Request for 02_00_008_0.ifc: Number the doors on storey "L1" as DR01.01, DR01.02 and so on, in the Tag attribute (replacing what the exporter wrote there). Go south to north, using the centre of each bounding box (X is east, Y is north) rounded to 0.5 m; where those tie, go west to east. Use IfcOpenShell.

First a look at what the model holds.

```python
import ifcopenshell
import ifcopenshell.util.element
import ifcopenshell.util.placement

model = ifcopenshell.open("02_00_008_0.ifc")
print(model.schema)
storey = next(s for s in model.by_type("IfcBuildingStorey") if s.Name == "L1")
doors = [e for e in ifcopenshell.util.element.get_decomposition(storey) if e.is_a("IfcDoor")]
for e in sorted(doors, key=lambda e: e.id()):
    origin = ifcopenshell.util.placement.get_local_placement(e.ObjectPlacement)[:3, 3]
    print(e.id(), e.Tag, e.Name, origin.round(2) + 0.0, sep=" | ")
```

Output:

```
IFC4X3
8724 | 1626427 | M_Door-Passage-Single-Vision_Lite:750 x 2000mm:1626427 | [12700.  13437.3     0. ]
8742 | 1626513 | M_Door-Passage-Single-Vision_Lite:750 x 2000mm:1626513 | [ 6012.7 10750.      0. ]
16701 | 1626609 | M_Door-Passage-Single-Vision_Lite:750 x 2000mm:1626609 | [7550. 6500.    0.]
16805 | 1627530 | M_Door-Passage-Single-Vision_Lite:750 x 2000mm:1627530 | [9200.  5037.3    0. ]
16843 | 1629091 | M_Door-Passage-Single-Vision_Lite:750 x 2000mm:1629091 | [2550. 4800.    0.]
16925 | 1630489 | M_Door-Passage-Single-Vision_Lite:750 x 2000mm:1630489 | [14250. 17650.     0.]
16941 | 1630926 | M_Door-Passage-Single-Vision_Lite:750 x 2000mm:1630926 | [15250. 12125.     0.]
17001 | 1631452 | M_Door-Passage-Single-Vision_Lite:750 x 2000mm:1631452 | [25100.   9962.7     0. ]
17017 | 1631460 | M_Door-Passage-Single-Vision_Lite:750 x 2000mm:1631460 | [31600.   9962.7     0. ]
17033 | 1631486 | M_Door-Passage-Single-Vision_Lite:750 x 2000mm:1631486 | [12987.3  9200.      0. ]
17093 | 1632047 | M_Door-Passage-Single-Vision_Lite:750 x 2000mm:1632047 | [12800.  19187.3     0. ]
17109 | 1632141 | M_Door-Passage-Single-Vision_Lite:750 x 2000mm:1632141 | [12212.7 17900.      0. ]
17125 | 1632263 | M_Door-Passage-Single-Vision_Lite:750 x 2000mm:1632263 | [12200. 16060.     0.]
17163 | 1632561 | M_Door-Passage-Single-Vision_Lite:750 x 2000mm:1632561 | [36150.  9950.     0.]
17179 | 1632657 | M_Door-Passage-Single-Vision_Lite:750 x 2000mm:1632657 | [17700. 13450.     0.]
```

```python
import ifcopenshell
import ifcopenshell.geom
import ifcopenshell.util.element
import ifcopenshell.util.shape

model = ifcopenshell.open("02_00_008_0.ifc")
settings = ifcopenshell.geom.settings()
settings.set("use-world-coords", True)


def centre(element):
    shape = ifcopenshell.geom.create_shape(settings, element)
    return ifcopenshell.util.shape.get_bbox_centroid(shape.geometry)


storey = next(s for s in model.by_type("IfcBuildingStorey") if s.Name == "L1")
doors = [e for e in ifcopenshell.util.element.get_decomposition(storey) if e.is_a("IfcDoor")]

# Insertion points can sit at a corner or the storey origin, so sort by the geometry (in metres).
centres = {e: centre(e) for e in doors}
doors.sort(key=lambda e: (round(centres[e][1] / 0.5), centres[e][0]))

for i, e in enumerate(doors, start=1):
    number = f"DR01.{i:02d}"
    e.Tag = number
    print(e.id(), number)

model.write("02_00_008_0_v2.ifc")
```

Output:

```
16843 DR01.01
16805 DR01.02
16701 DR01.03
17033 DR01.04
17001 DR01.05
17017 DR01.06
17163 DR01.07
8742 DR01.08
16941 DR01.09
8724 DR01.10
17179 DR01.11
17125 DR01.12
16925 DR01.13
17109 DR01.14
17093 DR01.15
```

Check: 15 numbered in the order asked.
